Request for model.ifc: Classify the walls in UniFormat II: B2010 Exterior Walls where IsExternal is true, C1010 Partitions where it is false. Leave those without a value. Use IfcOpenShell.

First a look at what the model holds.

```python
import ifcopenshell
import ifcopenshell.util.element

model = ifcopenshell.open("model.ifc")
print(model.schema)
print("classifications:", [c.Name for c in model.by_type("IfcClassification")])
values = [ifcopenshell.util.element.get_pset(e, "Pset_WallCommon", "IsExternal") for e in model.by_type("IfcWall")]
for value in (True, False, None):
    print("IsExternal", value, values.count(value))
```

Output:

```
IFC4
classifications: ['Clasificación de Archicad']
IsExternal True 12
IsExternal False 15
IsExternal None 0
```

```python
import ifcopenshell
import ifcopenshell.api.classification
import ifcopenshell.util.element

model = ifcopenshell.open("model.ifc")

system = ifcopenshell.api.classification.add_classification(model, classification="UniFormat II")

walls = model.by_type("IfcWall")
external = {e: ifcopenshell.util.element.get_pset(e, "Pset_WallCommon", "IsExternal") for e in walls}
for flag, code, name in ((True, "B2010", "Exterior Walls"), (False, "C1010", "Partitions")):
    products = [e for e in walls if external[e] is flag]
    ifcopenshell.api.classification.add_reference(
        model, products=products, classification=system, identification=code, name=name
    )
    print(code, len(products))

model.write("model_rev.ifc")
```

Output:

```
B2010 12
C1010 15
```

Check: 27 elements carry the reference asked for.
